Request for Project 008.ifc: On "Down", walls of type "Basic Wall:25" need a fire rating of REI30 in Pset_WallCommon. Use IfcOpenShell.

First a look at what the model holds.

```python
import ifcopenshell
import ifcopenshell.util.element

model = ifcopenshell.open("Project 008.ifc")
print(model.schema)
storey = next(s for s in model.by_type("IfcBuildingStorey") if s.Name == "Down")
walls = [e for e in ifcopenshell.util.element.get_decomposition(storey) if e.is_a("IfcWall")]
seen = {}
for e in walls:
    element_type = ifcopenshell.util.element.get_type(e)
    key = (element_type.Name if element_type != e and element_type else None, ifcopenshell.util.element.get_pset(e, "Pset_WallCommon", "FireRating"))
    seen[key] = seen.get(key, 0) + 1
for (name, value), count in sorted(seen.items(), key=str):
    print(count, "x", name, "|", value)
```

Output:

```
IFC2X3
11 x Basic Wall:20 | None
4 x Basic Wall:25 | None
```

```python
import ifcopenshell
import ifcopenshell.api.pset
import ifcopenshell.util.element

model = ifcopenshell.open("Project 008.ifc")

storey = next(s for s in model.by_type("IfcBuildingStorey") if s.Name == "Down")
walls = [e for e in ifcopenshell.util.element.get_decomposition(storey) if e.is_a("IfcWall")]

count = 0
for e in walls:
    element_type = ifcopenshell.util.element.get_type(e)
    if element_type in (None, e) or element_type.Name != "Basic Wall:25":
        continue
    # add_pset returns the element's existing set when there is one.
    pset = ifcopenshell.api.pset.add_pset(model, product=e, name="Pset_WallCommon")
    ifcopenshell.api.pset.edit_pset(model, pset=pset, properties={"FireRating": "REI30"})
    count += 1

print(count, "walls updated")

model.write("Project 008_rev.ifc")
```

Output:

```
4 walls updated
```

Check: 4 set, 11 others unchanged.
